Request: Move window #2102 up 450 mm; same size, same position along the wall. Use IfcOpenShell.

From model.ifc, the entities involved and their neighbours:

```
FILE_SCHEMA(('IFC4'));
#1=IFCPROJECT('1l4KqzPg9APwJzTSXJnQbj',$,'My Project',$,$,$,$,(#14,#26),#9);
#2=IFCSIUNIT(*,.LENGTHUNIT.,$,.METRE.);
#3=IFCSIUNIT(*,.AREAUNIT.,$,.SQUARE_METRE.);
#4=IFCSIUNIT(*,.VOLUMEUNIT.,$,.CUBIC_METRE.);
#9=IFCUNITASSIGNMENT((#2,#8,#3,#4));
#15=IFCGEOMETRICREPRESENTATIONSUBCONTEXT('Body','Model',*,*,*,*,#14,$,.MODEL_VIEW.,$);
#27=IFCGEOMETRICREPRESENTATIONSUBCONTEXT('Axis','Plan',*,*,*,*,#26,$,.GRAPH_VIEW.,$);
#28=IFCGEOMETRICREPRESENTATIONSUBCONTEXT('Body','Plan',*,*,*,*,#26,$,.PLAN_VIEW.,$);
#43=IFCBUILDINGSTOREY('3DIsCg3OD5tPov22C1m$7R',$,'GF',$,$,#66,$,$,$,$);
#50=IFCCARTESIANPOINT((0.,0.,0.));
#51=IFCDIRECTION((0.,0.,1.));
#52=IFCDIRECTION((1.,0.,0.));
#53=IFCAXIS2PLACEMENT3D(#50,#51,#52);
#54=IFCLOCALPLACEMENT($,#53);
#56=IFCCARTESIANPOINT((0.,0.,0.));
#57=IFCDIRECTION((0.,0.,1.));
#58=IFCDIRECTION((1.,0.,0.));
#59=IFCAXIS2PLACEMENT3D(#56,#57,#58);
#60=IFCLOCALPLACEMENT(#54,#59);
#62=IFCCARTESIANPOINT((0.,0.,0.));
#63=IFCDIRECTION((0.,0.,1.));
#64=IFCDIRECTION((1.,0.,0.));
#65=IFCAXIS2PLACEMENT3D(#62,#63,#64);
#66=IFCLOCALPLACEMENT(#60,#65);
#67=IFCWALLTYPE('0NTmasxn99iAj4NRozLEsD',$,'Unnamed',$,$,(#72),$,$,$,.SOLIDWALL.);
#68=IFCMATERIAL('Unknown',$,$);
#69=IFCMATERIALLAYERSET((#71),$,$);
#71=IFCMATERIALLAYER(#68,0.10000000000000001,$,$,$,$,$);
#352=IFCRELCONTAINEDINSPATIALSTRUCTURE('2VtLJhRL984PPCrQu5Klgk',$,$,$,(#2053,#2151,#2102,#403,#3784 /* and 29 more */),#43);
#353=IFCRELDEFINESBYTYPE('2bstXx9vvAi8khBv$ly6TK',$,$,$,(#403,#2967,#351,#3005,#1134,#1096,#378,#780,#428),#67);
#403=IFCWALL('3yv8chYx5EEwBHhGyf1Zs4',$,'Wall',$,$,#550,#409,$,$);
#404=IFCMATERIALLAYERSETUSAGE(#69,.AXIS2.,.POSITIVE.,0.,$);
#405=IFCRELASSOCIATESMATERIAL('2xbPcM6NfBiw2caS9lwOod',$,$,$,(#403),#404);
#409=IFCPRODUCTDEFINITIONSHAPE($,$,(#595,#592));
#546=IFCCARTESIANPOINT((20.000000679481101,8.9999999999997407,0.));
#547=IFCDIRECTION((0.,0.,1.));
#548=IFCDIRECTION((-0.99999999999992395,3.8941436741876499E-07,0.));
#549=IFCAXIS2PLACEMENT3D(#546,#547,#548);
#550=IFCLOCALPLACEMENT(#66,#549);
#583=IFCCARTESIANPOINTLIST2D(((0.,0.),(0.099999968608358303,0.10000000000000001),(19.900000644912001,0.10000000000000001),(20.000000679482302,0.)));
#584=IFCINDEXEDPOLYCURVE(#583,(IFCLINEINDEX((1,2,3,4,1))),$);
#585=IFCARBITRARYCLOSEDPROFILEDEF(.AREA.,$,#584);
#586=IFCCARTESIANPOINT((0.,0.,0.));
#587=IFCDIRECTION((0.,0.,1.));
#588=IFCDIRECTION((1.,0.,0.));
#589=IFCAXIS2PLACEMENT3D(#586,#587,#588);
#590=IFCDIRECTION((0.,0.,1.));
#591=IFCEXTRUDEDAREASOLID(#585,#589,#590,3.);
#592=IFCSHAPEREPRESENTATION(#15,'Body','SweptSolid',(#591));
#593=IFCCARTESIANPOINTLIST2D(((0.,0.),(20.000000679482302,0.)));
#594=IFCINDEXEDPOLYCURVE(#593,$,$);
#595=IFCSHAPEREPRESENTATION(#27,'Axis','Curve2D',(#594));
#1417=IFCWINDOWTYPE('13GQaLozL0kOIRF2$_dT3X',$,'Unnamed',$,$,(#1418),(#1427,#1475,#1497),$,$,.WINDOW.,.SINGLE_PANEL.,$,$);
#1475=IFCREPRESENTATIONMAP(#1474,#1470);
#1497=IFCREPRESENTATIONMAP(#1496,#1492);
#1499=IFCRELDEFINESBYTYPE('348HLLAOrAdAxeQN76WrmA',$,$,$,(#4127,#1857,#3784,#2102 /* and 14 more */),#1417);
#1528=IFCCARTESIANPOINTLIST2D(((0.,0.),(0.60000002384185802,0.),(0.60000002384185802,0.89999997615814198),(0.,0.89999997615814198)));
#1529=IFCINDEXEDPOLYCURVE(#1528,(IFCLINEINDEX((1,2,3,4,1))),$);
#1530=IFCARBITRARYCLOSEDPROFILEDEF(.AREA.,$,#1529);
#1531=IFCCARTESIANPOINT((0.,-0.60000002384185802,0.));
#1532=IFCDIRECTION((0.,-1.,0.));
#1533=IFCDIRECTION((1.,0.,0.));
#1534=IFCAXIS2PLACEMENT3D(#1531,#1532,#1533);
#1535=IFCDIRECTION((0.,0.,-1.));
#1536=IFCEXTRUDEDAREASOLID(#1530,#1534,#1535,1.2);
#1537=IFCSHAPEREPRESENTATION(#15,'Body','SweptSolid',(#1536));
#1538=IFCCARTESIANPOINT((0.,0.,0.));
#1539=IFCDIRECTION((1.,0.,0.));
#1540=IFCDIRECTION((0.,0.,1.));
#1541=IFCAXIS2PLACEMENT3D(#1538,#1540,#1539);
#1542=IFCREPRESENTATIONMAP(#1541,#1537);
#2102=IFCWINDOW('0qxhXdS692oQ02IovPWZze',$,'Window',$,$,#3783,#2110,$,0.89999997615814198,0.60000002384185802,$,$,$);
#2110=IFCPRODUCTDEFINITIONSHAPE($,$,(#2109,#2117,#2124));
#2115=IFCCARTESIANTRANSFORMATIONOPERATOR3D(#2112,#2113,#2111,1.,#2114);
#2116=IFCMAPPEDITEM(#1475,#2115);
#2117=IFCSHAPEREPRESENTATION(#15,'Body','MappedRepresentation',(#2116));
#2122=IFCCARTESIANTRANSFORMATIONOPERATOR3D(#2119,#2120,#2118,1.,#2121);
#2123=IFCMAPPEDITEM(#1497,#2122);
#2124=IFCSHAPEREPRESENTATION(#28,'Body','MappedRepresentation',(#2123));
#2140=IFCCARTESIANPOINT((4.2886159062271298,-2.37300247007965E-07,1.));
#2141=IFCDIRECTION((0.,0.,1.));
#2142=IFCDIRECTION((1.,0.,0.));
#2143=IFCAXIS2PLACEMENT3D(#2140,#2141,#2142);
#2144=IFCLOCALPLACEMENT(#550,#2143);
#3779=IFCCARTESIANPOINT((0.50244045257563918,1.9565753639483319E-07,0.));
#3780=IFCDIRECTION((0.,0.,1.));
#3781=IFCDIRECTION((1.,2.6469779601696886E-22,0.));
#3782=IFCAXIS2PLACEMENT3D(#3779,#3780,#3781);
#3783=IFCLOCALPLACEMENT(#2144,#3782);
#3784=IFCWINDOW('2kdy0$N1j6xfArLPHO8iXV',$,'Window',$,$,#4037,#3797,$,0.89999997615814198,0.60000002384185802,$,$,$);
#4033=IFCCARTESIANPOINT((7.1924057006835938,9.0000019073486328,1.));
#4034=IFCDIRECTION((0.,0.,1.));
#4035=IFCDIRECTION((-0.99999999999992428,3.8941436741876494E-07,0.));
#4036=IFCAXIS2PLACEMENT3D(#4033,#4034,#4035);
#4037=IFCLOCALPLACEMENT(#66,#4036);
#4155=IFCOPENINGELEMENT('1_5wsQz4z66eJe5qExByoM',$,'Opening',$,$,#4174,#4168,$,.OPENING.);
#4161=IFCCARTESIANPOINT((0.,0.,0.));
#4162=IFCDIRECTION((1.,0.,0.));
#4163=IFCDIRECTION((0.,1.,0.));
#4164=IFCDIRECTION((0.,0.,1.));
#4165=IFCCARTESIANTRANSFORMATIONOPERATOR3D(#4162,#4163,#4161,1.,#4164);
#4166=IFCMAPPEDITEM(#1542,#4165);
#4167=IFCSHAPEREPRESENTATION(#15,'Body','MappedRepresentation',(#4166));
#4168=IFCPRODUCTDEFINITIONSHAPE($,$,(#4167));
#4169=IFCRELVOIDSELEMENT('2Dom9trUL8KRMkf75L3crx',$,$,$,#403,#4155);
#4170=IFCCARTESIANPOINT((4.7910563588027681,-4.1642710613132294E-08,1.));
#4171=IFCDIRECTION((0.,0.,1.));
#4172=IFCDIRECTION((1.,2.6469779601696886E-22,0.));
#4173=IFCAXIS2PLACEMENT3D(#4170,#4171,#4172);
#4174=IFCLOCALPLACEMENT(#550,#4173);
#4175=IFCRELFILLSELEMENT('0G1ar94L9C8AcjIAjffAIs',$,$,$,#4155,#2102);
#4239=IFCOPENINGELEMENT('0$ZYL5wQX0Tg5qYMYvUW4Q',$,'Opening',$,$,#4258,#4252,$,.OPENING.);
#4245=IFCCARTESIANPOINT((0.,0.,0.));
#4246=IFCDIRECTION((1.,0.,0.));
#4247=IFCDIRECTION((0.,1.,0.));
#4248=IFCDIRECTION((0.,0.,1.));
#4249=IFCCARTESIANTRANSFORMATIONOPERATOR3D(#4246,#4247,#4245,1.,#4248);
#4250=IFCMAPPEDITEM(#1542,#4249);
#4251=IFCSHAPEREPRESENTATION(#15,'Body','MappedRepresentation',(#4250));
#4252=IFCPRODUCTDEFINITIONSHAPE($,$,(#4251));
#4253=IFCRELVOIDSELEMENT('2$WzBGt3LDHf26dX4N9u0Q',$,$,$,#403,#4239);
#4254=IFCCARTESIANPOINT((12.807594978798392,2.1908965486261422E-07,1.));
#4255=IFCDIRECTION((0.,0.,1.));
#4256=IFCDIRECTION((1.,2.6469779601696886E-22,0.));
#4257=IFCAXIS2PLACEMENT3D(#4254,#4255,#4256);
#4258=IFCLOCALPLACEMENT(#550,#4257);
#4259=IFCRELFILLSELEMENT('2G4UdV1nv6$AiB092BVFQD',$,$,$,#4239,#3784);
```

```python
import numpy as np
import ifcopenshell
import ifcopenshell.api.geometry
import ifcopenshell.util.placement
import ifcopenshell.util.unit

model = ifcopenshell.open("model.ifc")
unit_scale = ifcopenshell.util.unit.calculate_unit_scale(model)

window = model.by_id(2102)
opening = window.FillsVoids[0].RelatingOpeningElement
dz = 0.45 / unit_scale

shift = np.array([0.0, 0.0, dz])
# The window is not placed relative to its opening, so move both.
for product in (opening, window):
    matrix = ifcopenshell.util.placement.get_local_placement(product.ObjectPlacement)
    matrix[:3, 3] += shift
    ifcopenshell.api.geometry.edit_object_placement(model, product=product, matrix=matrix, is_si=False)

print(f"moved by {dz * unit_scale:+.3f} m")

model.write("model_edited.ifc")
```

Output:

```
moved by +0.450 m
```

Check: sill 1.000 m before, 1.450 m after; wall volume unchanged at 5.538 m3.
